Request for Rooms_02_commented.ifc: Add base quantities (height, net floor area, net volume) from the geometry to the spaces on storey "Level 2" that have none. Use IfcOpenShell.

First a look at what the model holds.

```python
import ifcopenshell
import ifcopenshell.util.element
import ifcopenshell.util.unit

model = ifcopenshell.open("Rooms_02_commented.ifc")
print(model.schema)
for unit_type in ("LENGTHUNIT", "AREAUNIT", "VOLUMEUNIT"):
    print(unit_type, ifcopenshell.util.unit.calculate_unit_scale(model, unit_type))
storey = next(s for s in model.by_type("IfcBuildingStorey") if s.Name == "Level 2")
spaces = [e for e in ifcopenshell.util.element.get_decomposition(storey) if e.is_a("IfcSpace")]
for e in sorted(spaces, key=lambda e: e.id()):
    print(e.id(), e.is_a(), e.Name, list(ifcopenshell.util.element.get_psets(e, qtos_only=True)), sep=" | ")
```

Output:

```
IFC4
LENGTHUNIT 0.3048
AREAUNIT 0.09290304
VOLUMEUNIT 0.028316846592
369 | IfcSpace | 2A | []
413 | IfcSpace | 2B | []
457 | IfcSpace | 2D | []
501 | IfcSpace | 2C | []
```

```python
import ifcopenshell
import ifcopenshell.api.pset
import ifcopenshell.geom
import ifcopenshell.util.element
import ifcopenshell.util.shape
import ifcopenshell.util.unit

model = ifcopenshell.open("Rooms_02_commented.ifc")
unit_scale = ifcopenshell.util.unit.calculate_unit_scale(model)
area_scale = ifcopenshell.util.unit.calculate_unit_scale(model, "AREAUNIT")
volume_scale = ifcopenshell.util.unit.calculate_unit_scale(model, "VOLUMEUNIT")
settings = ifcopenshell.geom.settings()

storey = next(s for s in model.by_type("IfcBuildingStorey") if s.Name == "Level 2")
spaces = [e for e in ifcopenshell.util.element.get_decomposition(storey) if e.is_a("IfcSpace")]

for e in sorted(spaces, key=lambda e: e.id()):
    if ifcopenshell.util.element.get_psets(e, qtos_only=True, should_inherit=False):
        continue
    # Geometry comes back in metres, in the element's own axes.
    shape = ifcopenshell.geom.create_shape(settings, e)
    values = {
        "Height": ifcopenshell.util.shape.get_z(shape.geometry) / unit_scale,
        "NetFloorArea": ifcopenshell.util.shape.get_footprint_area(shape.geometry) / area_scale,
        "NetVolume": ifcopenshell.util.shape.get_volume(shape.geometry) / volume_scale,
    }
    qto = ifcopenshell.api.pset.add_qto(model, product=e, name="Qto_SpaceBaseQuantities")
    ifcopenshell.api.pset.edit_qto(model, qto=qto, properties=values)
    print(e.id(), {k: round(v, 3) for k, v in values.items()})

model.write("Rooms_02_commented_v2.ifc")
```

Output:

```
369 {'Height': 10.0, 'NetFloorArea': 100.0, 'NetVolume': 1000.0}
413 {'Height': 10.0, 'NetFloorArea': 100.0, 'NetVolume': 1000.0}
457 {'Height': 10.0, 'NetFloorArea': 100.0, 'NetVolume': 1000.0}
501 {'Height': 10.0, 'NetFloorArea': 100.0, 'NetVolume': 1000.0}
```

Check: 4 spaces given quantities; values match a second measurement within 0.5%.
